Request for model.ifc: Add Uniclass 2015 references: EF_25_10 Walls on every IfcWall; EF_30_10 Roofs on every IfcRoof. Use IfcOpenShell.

First a look at what the model holds.

```python
import ifcopenshell

model = ifcopenshell.open("model.ifc")
print(model.schema)
print("classifications:", [c.Name for c in model.by_type("IfcClassification")])
for ifc_class in ("IfcDoor", "IfcRoof", "IfcStair", "IfcWall", "IfcWindow"):
    print(ifc_class, len(model.by_type(ifc_class)))
```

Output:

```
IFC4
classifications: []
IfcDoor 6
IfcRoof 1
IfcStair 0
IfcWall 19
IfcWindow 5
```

```python
import ifcopenshell
import ifcopenshell.api.classification

model = ifcopenshell.open("model.ifc")

system = ifcopenshell.api.classification.add_classification(model, classification="Uniclass 2015")

codes = {
    "IfcWall": ("EF_25_10", "Walls"),
    "IfcRoof": ("EF_30_10", "Roofs"),
}
for ifc_class, (code, name) in codes.items():
    products = model.by_type(ifc_class)
    ifcopenshell.api.classification.add_reference(
        model, products=products, classification=system, identification=code, name=name
    )
    print(code, len(products))

model.write("model_v2.ifc")
```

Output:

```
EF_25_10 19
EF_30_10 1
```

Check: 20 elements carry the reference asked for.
